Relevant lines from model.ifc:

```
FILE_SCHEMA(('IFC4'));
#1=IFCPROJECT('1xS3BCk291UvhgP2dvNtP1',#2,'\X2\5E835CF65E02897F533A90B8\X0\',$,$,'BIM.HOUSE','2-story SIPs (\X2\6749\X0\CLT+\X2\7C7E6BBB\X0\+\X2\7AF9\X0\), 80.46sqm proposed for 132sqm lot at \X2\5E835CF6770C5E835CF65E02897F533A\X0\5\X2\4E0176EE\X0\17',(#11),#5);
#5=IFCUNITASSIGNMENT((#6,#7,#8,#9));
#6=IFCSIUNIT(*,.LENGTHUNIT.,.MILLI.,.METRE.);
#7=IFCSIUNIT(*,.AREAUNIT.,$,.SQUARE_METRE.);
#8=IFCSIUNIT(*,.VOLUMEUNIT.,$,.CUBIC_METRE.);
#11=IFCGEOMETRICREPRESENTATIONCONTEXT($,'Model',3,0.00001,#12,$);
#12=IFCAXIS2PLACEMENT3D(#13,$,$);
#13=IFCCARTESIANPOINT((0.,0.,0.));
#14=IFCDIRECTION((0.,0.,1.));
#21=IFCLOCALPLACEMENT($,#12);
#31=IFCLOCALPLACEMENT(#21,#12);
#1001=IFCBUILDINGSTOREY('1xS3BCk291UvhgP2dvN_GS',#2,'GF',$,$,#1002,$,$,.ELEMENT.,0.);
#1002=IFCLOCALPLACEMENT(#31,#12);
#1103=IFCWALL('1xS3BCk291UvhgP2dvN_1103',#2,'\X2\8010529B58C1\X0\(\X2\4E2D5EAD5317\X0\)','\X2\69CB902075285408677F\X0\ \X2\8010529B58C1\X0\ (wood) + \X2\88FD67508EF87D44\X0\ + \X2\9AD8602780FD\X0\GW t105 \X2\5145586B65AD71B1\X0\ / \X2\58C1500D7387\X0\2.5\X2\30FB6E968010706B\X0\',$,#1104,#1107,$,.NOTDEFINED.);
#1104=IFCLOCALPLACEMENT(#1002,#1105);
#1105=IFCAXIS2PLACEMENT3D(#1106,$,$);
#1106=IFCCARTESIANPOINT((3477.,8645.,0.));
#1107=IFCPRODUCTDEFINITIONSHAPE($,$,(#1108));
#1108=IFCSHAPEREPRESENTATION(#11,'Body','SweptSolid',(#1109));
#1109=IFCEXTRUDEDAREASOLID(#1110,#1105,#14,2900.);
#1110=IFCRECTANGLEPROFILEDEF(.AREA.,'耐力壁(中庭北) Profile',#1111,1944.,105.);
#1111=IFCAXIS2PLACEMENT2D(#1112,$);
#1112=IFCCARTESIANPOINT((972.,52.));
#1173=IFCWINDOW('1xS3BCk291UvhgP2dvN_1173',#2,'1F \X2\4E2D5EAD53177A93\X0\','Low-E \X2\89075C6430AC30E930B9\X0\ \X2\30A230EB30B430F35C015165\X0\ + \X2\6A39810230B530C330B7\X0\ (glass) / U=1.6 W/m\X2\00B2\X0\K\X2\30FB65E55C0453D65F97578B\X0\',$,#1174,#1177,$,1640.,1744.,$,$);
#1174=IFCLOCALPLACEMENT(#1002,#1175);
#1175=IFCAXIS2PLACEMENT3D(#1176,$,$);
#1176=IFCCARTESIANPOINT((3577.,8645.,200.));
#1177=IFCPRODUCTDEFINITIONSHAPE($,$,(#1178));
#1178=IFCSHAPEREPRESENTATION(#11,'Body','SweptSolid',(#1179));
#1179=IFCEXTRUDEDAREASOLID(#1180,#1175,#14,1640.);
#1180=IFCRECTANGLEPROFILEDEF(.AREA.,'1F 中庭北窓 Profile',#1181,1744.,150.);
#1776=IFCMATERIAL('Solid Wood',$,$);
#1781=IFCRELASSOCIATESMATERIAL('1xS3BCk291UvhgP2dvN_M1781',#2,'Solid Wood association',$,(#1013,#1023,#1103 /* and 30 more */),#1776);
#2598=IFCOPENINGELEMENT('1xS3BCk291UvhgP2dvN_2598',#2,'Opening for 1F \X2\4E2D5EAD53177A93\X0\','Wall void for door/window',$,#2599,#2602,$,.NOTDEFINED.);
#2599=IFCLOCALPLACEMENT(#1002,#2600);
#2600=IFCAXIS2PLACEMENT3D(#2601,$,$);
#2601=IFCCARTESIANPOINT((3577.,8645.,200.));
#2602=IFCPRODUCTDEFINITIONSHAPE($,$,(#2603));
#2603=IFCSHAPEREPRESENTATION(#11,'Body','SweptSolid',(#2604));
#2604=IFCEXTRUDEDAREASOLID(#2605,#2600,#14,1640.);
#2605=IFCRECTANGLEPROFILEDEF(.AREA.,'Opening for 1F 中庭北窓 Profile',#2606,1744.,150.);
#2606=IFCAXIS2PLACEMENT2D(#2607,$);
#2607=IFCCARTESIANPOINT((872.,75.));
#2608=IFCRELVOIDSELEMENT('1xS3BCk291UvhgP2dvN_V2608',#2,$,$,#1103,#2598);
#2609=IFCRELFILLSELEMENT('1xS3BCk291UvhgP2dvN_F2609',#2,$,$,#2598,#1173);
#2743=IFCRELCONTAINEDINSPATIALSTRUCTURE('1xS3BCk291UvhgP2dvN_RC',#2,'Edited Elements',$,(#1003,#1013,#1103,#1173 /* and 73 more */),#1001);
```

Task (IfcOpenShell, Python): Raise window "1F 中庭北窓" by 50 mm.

```python
import numpy as np
import ifcopenshell
import ifcopenshell.api.geometry
import ifcopenshell.util.placement
import ifcopenshell.util.unit

model = ifcopenshell.open("model.ifc")
unit_scale = ifcopenshell.util.unit.calculate_unit_scale(model)

window = model.by_id(1173)
opening = window.FillsVoids[0].RelatingOpeningElement
dz = 50.0

shift = np.array([0.0, 0.0, dz])
# The window is not placed relative to its opening, so move both.
for product in (opening, window):
    matrix = ifcopenshell.util.placement.get_local_placement(product.ObjectPlacement)
    matrix[:3, 3] += shift
    ifcopenshell.api.geometry.edit_object_placement(model, product=product, matrix=matrix, is_si=False)

print(f"moved by {dz * unit_scale:+.3f} m")

model.write("model_updated.ifc")
```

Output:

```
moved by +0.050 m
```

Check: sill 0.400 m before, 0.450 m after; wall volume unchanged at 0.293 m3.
